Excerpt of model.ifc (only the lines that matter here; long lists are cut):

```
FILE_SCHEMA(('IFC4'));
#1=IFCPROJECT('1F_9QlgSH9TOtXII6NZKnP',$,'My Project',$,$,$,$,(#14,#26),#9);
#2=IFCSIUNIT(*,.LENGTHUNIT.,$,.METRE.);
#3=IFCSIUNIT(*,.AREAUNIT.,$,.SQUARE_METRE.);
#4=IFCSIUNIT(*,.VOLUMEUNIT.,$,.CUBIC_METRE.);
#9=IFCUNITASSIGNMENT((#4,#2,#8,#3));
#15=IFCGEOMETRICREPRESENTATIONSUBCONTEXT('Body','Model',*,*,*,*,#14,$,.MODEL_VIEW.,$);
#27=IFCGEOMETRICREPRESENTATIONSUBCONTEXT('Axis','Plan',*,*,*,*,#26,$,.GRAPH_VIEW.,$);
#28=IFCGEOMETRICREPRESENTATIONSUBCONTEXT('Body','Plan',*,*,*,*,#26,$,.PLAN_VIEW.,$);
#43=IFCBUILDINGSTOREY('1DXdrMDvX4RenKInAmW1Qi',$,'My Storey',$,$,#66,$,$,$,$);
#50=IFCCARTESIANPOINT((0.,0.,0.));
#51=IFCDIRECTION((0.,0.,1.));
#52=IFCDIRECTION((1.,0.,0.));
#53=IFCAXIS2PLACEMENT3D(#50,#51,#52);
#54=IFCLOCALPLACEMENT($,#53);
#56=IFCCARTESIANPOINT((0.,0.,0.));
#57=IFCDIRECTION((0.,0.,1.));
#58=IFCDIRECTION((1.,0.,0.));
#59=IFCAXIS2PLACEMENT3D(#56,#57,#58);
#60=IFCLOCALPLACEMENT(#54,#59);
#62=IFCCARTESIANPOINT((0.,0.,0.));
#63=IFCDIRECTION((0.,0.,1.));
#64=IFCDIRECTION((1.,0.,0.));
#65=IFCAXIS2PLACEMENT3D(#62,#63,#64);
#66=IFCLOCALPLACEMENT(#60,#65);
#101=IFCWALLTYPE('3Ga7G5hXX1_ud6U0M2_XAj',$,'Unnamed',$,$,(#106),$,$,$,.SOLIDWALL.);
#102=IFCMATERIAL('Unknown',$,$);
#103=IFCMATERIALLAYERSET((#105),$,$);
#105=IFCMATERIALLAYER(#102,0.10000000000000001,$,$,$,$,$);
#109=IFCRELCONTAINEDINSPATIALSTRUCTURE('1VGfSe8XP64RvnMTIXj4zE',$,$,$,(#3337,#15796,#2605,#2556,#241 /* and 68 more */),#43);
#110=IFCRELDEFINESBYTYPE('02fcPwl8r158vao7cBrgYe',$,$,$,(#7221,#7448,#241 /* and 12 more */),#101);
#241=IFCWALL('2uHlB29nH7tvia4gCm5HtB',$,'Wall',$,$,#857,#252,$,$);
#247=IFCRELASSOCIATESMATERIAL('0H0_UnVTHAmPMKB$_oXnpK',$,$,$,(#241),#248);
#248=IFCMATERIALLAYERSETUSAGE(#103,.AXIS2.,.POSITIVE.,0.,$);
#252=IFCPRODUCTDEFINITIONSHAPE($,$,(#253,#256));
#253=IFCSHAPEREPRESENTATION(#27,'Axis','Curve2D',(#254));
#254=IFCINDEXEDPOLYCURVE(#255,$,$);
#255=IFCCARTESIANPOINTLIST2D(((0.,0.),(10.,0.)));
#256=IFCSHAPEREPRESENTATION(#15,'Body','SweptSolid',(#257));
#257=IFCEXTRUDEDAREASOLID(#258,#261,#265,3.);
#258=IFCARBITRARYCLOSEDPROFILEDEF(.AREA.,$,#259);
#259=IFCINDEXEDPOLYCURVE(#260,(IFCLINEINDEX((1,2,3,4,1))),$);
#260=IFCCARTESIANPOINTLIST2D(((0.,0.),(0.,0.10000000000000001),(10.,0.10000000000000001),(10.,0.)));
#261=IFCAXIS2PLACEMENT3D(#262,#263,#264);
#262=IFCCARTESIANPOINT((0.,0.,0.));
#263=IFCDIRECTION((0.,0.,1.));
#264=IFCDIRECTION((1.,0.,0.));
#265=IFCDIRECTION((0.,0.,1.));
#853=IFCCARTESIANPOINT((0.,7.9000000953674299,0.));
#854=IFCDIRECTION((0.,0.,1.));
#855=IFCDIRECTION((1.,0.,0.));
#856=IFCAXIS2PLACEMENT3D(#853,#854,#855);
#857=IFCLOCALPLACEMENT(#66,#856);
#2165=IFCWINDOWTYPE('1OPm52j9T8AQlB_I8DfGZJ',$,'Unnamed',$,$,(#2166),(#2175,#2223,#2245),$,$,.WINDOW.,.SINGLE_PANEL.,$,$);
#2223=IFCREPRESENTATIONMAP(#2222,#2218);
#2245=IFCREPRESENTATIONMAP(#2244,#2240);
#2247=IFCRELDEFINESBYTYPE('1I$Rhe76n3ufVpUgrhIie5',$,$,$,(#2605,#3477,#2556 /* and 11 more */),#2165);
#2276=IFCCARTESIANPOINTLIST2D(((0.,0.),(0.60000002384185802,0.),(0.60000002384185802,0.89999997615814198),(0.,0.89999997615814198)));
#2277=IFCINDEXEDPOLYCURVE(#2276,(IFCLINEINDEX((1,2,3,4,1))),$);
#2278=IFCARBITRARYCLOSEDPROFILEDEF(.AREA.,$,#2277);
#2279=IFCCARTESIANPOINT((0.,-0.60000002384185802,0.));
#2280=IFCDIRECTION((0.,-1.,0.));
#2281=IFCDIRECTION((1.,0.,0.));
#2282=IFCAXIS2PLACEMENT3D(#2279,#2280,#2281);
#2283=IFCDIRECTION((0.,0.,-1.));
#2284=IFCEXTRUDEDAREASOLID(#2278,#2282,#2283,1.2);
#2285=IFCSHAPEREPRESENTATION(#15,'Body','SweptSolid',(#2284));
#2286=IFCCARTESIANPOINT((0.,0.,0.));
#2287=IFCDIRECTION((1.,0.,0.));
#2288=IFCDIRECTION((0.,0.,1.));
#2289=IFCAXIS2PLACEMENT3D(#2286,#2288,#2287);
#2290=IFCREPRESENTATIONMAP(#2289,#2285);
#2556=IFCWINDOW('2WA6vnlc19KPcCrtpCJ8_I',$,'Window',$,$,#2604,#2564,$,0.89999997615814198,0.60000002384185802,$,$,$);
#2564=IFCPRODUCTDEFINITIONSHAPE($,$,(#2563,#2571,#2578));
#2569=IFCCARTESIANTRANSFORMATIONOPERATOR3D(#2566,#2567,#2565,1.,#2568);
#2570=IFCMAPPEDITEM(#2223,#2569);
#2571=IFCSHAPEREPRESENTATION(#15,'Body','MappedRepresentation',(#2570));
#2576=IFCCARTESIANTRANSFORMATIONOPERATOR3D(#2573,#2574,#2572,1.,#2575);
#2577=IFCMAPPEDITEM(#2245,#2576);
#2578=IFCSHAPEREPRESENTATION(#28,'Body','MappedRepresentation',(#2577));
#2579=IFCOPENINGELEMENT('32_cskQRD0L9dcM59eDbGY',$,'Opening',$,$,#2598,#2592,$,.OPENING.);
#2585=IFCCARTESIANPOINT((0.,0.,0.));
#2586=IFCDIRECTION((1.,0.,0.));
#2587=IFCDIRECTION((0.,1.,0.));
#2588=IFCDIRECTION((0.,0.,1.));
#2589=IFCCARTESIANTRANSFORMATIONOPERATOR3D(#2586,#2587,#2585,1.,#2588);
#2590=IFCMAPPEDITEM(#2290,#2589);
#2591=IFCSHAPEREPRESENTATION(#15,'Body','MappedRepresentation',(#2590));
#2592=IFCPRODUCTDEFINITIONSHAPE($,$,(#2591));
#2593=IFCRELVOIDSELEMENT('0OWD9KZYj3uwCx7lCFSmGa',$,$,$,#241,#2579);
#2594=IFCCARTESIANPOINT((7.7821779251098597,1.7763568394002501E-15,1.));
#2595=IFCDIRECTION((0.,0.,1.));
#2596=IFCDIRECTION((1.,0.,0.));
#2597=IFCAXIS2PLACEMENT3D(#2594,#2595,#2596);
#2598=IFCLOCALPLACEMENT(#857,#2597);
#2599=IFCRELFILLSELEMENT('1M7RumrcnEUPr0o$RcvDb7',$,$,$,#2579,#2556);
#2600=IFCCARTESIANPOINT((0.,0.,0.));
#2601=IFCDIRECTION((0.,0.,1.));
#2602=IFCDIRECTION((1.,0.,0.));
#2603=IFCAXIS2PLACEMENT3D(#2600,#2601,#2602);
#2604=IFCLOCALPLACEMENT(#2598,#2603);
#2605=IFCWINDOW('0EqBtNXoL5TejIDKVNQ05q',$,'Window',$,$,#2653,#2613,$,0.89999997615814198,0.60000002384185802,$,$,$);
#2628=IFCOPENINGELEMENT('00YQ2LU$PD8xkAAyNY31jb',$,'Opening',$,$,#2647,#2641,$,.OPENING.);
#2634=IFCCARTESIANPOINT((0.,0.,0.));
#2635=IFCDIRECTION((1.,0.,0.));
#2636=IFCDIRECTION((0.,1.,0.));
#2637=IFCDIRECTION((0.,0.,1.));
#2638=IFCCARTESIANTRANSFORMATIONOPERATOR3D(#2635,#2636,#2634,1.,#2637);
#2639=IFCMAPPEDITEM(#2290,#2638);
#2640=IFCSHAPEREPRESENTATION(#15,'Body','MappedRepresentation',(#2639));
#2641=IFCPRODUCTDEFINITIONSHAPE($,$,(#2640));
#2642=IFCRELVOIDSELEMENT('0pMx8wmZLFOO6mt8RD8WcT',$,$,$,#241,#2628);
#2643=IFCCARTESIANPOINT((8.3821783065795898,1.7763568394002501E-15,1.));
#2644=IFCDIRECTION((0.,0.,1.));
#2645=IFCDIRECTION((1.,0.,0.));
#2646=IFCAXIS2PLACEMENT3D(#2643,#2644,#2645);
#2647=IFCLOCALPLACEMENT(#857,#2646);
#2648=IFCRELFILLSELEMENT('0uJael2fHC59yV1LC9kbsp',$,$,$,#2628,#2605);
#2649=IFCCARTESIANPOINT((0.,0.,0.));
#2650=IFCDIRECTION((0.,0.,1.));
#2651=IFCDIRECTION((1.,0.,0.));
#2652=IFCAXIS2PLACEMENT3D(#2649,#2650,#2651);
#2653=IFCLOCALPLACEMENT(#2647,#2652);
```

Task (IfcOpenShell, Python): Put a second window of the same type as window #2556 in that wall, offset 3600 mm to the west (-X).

```python
import ifcopenshell
import ifcopenshell.api.feature
import ifcopenshell.api.geometry
import ifcopenshell.api.root
import ifcopenshell.geom
import ifcopenshell.util.element
import ifcopenshell.util.placement
import ifcopenshell.util.shape

model = ifcopenshell.open("model.ifc")
settings = ifcopenshell.geom.settings()


def volume(element):
    """Net volume in cubic metres, openings subtracted."""
    shape = ifcopenshell.geom.create_shape(settings, element)
    return ifcopenshell.util.shape.get_volume(shape.geometry)


window = model.by_id(2556)
opening = window.FillsVoids[0].RelatingOpeningElement
wall = opening.VoidsElements[0].RelatingBuildingElement
before = volume(wall)
shift = ifcopenshell.util.placement.get_local_placement(wall.ObjectPlacement)[:3, 0] * -3.6

# copy_class copies the void relationship, type, container and properties, but no geometry.
new_opening = ifcopenshell.api.root.copy_class(model, product=opening)
new_opening.Representation = ifcopenshell.util.element.copy_deep(
    model, opening.Representation, exclude=["IfcGeometricRepresentationContext", "IfcRepresentationMap"]
)
new_window = ifcopenshell.api.root.copy_class(model, product=window)
new_window.Representation = ifcopenshell.util.element.copy_deep(
    model, window.Representation, exclude=["IfcGeometricRepresentationContext", "IfcRepresentationMap"]
)
ifcopenshell.api.feature.add_filling(model, opening=new_opening, element=new_window)

for old, new in ((opening, new_opening), (window, new_window)):
    matrix = ifcopenshell.util.placement.get_local_placement(old.ObjectPlacement)
    matrix[:3, 3] += shift
    ifcopenshell.api.geometry.edit_object_placement(model, product=new, matrix=matrix, is_si=False)

after = volume(wall)

print(f"wall volume {before:.3f} -> {after:.3f} m3")

model.write("model-out.ifc")
```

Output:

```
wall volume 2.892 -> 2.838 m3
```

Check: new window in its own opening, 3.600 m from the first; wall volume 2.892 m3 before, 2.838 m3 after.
